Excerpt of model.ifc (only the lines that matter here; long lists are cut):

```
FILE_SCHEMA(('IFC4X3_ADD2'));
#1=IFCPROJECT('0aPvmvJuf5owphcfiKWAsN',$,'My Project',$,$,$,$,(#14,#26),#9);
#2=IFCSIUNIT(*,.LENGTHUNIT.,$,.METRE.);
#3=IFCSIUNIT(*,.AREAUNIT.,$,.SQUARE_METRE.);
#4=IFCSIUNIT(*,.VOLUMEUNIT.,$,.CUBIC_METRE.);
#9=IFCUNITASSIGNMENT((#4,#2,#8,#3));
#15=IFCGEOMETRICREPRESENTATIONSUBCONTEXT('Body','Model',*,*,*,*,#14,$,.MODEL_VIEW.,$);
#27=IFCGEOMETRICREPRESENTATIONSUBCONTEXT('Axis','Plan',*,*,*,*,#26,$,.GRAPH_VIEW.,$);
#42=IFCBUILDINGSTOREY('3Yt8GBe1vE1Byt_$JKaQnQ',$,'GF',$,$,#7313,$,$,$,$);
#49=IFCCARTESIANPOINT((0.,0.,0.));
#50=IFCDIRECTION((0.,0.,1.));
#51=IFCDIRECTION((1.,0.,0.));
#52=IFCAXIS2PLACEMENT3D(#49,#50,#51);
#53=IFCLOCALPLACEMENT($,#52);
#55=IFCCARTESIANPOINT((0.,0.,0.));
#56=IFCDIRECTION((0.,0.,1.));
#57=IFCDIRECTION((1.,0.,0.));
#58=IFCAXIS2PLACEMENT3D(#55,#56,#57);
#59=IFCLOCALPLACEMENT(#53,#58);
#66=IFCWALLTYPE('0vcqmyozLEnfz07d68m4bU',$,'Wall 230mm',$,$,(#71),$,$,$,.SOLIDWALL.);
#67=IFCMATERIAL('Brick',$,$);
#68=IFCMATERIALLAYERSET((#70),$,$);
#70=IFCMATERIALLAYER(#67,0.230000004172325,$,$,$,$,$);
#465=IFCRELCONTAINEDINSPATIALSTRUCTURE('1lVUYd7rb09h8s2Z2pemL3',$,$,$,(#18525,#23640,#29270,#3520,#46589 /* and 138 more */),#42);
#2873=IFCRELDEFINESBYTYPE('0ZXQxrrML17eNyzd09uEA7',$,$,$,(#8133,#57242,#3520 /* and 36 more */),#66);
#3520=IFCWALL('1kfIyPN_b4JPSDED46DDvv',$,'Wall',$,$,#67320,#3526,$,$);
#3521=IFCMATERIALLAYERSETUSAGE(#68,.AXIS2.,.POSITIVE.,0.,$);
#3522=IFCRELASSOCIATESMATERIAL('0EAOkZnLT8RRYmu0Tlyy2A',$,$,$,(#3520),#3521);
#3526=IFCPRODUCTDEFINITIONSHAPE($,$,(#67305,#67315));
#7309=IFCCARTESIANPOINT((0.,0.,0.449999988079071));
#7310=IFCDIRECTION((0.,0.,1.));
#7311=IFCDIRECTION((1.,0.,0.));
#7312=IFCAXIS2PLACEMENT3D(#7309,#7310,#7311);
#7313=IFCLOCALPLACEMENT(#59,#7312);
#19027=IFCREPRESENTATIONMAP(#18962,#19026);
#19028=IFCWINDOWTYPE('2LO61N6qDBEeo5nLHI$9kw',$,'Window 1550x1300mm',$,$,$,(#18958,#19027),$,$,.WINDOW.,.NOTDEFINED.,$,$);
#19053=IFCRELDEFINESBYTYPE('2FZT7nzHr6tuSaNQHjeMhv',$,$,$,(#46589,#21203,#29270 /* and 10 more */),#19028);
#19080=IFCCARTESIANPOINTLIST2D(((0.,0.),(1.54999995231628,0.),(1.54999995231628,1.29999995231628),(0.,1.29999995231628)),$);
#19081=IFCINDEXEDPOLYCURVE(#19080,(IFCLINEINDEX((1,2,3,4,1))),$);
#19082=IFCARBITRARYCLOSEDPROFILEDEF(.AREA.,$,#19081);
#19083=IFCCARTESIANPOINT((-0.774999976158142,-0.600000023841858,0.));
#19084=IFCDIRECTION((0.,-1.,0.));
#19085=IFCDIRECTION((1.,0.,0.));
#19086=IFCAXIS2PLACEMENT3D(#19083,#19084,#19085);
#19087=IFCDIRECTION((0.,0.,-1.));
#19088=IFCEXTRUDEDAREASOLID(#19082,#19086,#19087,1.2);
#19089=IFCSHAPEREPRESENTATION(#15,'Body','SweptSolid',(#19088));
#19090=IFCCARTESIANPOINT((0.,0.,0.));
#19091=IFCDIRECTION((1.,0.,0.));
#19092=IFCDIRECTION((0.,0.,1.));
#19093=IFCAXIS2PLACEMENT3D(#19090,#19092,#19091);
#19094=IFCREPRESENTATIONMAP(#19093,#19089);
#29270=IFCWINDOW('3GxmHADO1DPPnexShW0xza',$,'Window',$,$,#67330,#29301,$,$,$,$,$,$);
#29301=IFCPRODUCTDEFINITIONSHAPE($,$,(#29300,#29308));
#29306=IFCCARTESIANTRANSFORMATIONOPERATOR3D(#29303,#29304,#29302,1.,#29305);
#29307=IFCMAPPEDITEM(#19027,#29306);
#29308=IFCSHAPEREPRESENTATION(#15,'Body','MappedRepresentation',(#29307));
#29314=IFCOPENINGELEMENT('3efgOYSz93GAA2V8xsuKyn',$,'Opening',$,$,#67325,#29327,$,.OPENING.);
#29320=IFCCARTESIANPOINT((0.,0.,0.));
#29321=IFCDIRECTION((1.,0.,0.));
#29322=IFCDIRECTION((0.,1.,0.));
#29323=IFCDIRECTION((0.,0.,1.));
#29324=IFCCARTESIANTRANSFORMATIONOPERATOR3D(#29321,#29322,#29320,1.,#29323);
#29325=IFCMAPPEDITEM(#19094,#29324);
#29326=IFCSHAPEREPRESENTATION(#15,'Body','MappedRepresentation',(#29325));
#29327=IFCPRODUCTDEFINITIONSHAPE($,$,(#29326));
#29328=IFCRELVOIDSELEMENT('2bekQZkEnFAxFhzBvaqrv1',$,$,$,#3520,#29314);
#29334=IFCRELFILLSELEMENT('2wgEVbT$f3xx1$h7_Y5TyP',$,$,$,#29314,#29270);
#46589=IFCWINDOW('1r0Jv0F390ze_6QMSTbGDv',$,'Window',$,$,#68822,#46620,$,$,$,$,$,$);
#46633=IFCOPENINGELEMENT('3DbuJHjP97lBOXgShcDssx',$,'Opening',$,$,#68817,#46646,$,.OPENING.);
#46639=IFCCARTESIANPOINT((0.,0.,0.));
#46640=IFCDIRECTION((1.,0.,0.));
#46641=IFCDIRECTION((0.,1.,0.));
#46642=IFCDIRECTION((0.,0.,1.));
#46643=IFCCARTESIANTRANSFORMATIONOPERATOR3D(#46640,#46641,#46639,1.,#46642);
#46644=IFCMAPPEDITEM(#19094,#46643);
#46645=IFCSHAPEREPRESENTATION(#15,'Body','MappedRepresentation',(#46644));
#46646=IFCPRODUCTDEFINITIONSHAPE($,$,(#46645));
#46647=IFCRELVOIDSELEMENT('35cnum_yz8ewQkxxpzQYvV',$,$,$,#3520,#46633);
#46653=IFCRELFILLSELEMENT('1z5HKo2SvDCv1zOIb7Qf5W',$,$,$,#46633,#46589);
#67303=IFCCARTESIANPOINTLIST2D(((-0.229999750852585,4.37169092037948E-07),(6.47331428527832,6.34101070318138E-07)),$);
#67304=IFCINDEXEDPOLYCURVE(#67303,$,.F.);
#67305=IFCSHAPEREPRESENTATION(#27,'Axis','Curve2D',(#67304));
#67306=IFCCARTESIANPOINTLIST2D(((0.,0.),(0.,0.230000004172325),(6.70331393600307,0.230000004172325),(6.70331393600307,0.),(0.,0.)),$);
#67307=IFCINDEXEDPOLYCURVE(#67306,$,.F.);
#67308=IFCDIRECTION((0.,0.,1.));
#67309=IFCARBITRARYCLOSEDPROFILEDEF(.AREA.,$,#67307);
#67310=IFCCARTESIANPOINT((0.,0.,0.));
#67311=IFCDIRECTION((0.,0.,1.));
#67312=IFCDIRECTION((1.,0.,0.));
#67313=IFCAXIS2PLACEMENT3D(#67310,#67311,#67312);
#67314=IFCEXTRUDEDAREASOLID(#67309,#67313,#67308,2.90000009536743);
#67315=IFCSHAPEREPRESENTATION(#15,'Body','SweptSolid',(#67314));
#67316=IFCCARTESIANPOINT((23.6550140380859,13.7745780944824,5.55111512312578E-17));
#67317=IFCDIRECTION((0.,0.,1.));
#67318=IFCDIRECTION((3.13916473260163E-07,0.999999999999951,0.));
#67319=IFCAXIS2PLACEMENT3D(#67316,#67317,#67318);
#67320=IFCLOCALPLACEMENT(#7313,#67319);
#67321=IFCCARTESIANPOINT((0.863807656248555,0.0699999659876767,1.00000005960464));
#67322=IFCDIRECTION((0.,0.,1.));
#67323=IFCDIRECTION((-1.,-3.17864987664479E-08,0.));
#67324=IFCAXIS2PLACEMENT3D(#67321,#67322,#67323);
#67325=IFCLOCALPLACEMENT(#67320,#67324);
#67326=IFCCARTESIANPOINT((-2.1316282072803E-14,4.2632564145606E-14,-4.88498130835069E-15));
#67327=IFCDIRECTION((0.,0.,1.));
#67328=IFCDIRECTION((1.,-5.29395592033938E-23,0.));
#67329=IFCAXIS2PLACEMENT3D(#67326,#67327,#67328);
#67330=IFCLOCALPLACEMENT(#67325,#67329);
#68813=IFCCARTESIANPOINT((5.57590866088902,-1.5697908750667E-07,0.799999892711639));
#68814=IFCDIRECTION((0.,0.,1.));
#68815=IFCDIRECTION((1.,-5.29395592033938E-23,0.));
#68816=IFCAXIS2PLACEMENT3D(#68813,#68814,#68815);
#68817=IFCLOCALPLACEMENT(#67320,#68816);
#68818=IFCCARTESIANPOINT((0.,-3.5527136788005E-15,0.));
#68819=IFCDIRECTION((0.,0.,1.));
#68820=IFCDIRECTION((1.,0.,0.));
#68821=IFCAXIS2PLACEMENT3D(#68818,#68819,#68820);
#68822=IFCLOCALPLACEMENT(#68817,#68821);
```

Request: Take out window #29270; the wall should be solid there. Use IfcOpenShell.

```python
import ifcopenshell
import ifcopenshell.api.feature
import ifcopenshell.api.root
import ifcopenshell.geom
import ifcopenshell.util.shape

model = ifcopenshell.open("model.ifc")
settings = ifcopenshell.geom.settings()


def volume(element):
    """Net volume in cubic metres, openings subtracted."""
    shape = ifcopenshell.geom.create_shape(settings, element)
    return ifcopenshell.util.shape.get_volume(shape.geometry)


window = model.by_guid("3GxmHADO1DPPnexShW0xza")
opening = window.FillsVoids[0].RelatingOpeningElement
wall = opening.VoidsElements[0].RelatingBuildingElement
before = volume(wall)

ifcopenshell.api.root.remove_product(model, product=window)
ifcopenshell.api.feature.remove_feature(model, feature=opening)

after = volume(wall)

print(f"wall volume {before:.3f} -> {after:.3f} m3")

model.write("model-out.ifc")
```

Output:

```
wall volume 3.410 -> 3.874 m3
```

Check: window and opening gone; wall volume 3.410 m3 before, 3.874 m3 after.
